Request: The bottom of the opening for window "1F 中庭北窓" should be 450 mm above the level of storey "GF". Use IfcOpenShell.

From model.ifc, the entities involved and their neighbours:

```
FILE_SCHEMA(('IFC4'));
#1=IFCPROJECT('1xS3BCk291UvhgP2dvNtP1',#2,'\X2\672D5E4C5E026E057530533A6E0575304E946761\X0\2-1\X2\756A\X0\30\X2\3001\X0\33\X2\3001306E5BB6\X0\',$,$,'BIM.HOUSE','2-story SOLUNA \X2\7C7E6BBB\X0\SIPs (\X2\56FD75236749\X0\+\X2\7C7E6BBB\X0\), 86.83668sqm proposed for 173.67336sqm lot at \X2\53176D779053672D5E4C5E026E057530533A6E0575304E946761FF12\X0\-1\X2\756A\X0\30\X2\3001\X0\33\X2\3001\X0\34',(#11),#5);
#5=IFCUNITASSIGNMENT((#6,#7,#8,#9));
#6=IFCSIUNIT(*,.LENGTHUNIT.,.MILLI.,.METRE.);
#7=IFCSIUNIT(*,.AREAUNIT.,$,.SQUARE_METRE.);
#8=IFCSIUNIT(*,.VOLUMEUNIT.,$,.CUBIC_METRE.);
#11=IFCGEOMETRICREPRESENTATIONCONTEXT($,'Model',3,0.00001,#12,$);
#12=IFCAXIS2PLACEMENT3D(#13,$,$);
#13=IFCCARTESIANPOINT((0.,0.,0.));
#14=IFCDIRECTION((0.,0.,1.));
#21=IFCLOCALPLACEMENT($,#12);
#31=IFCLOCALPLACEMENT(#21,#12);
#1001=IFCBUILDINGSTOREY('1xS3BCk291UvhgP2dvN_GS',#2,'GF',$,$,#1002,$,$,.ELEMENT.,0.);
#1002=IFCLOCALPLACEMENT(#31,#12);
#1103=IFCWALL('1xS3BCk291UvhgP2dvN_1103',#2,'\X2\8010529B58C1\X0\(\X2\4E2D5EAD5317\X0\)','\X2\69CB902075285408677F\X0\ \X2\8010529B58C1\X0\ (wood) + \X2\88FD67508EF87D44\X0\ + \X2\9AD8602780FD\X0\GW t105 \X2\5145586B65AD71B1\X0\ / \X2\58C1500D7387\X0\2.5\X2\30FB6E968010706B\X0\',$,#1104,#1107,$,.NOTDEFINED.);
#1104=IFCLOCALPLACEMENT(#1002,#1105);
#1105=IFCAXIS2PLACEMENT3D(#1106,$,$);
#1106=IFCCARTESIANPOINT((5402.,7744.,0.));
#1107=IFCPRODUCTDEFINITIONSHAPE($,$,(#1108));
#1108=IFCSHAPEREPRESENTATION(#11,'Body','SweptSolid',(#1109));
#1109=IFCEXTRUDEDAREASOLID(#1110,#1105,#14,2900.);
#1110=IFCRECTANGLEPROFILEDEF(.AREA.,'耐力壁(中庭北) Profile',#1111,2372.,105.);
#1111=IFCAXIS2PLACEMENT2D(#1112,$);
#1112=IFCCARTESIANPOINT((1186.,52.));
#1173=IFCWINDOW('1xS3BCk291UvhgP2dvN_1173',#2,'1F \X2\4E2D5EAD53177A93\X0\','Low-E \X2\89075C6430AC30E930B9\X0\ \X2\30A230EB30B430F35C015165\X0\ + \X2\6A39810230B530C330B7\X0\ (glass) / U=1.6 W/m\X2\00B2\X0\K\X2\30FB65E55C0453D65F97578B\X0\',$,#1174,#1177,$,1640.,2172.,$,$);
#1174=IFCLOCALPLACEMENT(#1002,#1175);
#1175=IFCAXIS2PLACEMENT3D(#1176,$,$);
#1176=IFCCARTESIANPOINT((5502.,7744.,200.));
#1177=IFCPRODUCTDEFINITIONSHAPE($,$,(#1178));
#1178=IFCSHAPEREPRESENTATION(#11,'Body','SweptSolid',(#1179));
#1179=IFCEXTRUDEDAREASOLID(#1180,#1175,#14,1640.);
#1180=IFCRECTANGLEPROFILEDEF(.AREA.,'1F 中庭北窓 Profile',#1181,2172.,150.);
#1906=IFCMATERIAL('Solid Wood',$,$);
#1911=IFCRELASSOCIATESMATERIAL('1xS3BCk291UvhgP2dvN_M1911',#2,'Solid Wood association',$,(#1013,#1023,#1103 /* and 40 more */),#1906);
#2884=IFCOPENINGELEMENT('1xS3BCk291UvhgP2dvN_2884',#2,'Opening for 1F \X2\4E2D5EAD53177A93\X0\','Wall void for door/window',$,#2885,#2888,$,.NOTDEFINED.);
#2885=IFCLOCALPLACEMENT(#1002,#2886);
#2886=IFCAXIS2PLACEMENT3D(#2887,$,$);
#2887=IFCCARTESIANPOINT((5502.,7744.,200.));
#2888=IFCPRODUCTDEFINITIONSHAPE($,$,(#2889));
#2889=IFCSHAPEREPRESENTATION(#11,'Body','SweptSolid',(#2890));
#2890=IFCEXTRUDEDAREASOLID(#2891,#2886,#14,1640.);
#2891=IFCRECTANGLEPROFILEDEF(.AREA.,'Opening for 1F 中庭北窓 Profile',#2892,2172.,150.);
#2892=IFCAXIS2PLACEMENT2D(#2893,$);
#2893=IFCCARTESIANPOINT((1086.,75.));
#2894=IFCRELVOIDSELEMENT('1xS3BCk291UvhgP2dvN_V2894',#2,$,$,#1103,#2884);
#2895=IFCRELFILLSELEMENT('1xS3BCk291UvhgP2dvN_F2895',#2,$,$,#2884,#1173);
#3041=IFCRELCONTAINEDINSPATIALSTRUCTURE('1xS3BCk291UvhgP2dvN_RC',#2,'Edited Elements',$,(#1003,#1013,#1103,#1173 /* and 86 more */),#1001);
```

```python
import numpy as np
import ifcopenshell
import ifcopenshell.api.geometry
import ifcopenshell.geom
import ifcopenshell.util.element
import ifcopenshell.util.placement
import ifcopenshell.util.shape
import ifcopenshell.util.unit

model = ifcopenshell.open("model.ifc")
unit_scale = ifcopenshell.util.unit.calculate_unit_scale(model)

window = model.by_guid("1xS3BCk291UvhgP2dvN_1173")
opening = window.FillsVoids[0].RelatingOpeningElement
storey = ifcopenshell.util.element.get_container(window, ifc_class="IfcBuildingStorey")
level = ifcopenshell.util.placement.get_local_placement(storey.ObjectPlacement)[2, 3]

# The opening's origin need not be at the sill, so measure its lowest point.
shape = ifcopenshell.geom.create_shape(ifcopenshell.geom.settings(), opening)
bottom = ifcopenshell.util.shape.get_shape_bottom_elevation(shape, shape.geometry) / unit_scale
dz = level + 0.45 / unit_scale - bottom

shift = np.array([0.0, 0.0, dz])
# The window is not placed relative to its opening, so move both.
for product in (opening, window):
    matrix = ifcopenshell.util.placement.get_local_placement(product.ObjectPlacement)
    matrix[:3, 3] += shift
    ifcopenshell.api.geometry.edit_object_placement(model, product=product, matrix=matrix, is_si=False)

print(f"moved by {dz * unit_scale:+.3f} m")

model.write("model_rev.ifc")
```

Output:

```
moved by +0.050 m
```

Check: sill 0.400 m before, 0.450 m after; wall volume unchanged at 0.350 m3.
